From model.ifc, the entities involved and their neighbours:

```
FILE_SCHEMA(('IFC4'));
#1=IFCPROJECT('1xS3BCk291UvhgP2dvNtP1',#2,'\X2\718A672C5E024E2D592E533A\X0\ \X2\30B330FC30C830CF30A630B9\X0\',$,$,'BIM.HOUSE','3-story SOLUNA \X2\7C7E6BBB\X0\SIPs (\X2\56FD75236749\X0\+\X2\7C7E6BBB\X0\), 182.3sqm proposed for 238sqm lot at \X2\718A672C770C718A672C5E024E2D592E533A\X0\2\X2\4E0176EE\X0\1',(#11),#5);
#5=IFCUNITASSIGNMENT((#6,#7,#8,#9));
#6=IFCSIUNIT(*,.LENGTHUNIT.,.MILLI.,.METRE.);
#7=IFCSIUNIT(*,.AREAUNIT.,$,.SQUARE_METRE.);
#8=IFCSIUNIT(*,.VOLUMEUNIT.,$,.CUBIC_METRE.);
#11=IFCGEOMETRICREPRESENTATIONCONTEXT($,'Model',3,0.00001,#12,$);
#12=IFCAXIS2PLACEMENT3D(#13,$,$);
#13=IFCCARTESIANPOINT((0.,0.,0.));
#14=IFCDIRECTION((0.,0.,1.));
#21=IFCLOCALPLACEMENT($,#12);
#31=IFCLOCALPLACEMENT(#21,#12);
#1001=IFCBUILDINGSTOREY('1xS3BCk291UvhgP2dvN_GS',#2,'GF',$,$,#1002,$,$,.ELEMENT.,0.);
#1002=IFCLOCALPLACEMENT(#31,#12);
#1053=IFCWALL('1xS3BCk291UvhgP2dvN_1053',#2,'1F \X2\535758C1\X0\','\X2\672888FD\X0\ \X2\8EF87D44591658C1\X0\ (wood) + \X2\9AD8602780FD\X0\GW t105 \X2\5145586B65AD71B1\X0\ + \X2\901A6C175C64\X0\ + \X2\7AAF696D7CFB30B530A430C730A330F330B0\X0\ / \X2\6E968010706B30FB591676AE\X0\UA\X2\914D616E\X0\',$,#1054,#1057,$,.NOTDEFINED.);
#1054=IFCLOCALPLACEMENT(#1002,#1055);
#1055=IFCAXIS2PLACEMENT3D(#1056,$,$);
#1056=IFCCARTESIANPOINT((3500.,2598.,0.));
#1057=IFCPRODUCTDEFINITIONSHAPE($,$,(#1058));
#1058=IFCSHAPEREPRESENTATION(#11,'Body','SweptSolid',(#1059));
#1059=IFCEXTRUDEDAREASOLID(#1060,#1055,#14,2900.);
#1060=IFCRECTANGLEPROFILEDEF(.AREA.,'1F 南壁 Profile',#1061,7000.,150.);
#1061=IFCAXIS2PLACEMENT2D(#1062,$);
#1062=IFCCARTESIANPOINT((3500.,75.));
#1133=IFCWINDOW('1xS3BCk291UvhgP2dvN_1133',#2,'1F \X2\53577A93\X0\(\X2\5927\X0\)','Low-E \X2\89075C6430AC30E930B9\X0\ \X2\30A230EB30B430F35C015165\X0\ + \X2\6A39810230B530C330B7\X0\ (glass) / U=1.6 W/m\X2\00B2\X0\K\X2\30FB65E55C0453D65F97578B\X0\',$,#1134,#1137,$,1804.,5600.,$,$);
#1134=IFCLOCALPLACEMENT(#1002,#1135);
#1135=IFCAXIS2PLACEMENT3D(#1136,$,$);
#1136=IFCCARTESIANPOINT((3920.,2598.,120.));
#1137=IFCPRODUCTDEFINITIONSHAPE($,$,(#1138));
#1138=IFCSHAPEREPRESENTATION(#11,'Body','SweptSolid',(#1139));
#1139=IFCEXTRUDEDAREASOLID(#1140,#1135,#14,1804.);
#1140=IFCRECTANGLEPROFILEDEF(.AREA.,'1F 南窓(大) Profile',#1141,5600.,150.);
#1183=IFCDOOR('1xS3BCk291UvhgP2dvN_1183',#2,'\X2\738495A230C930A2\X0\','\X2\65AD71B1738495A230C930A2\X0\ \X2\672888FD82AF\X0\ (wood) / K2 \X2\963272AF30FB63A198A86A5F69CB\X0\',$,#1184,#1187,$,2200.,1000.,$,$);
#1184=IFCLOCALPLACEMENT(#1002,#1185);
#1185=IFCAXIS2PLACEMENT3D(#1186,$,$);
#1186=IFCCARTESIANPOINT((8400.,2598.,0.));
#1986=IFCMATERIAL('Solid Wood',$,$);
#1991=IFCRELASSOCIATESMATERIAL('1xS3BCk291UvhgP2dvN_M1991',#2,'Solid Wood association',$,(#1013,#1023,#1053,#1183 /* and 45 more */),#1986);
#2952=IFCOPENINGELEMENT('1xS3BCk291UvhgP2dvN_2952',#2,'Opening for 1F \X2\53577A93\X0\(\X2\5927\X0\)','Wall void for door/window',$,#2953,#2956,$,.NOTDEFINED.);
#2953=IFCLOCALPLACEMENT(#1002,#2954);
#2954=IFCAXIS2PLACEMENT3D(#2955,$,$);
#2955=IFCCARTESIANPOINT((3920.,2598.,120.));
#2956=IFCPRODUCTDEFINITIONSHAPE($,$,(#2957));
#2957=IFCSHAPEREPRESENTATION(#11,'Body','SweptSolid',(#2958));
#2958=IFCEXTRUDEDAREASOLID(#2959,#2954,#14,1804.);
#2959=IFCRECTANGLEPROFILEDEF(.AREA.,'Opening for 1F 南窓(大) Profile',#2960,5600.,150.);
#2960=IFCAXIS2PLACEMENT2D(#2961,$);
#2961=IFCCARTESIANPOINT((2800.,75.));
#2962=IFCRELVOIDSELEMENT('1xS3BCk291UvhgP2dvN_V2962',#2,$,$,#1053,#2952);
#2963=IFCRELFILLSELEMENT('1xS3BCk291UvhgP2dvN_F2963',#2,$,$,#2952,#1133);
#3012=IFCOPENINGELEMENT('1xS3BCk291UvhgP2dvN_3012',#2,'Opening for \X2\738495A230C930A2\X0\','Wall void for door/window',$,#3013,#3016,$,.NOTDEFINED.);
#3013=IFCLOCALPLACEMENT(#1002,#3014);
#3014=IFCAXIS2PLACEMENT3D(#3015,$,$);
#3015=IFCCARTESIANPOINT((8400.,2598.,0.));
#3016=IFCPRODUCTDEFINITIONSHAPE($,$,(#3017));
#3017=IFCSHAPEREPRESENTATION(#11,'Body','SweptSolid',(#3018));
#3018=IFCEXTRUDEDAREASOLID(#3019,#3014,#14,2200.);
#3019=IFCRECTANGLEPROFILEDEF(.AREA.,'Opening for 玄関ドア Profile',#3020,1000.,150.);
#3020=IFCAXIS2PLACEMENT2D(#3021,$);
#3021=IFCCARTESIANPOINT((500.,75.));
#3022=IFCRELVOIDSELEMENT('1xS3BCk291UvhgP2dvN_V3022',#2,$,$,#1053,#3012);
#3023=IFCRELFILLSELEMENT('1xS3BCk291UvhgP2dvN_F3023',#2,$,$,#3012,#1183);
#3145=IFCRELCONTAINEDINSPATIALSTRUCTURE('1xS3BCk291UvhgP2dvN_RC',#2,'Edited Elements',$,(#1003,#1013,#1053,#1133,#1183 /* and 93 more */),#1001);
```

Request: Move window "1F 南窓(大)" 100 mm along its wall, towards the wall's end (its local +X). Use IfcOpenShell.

```python
import ifcopenshell
import ifcopenshell.api.geometry
import ifcopenshell.util.placement

model = ifcopenshell.open("model.ifc")

window = model.by_guid("1xS3BCk291UvhgP2dvN_1133")
opening = window.FillsVoids[0].RelatingOpeningElement
wall = opening.VoidsElements[0].RelatingBuildingElement

wall_matrix = ifcopenshell.util.placement.get_local_placement(wall.ObjectPlacement)
shift = wall_matrix[:3, 0] * 100.0
before = ifcopenshell.util.placement.get_local_placement(window.ObjectPlacement)[:3, 3].copy()

# The window is not placed relative to its opening, so move both.
for product in (opening, window):
    matrix = ifcopenshell.util.placement.get_local_placement(product.ObjectPlacement)
    matrix[:3, 3] += shift
    ifcopenshell.api.geometry.edit_object_placement(model, product=product, matrix=matrix, is_si=False)

after = ifcopenshell.util.placement.get_local_placement(window.ObjectPlacement)[:3, 3]
print("window moved by", (after - before).round(3) + 0.0)

model.write("model_v2.ifc")
```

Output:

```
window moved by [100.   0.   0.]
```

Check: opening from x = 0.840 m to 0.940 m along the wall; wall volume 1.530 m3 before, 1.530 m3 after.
